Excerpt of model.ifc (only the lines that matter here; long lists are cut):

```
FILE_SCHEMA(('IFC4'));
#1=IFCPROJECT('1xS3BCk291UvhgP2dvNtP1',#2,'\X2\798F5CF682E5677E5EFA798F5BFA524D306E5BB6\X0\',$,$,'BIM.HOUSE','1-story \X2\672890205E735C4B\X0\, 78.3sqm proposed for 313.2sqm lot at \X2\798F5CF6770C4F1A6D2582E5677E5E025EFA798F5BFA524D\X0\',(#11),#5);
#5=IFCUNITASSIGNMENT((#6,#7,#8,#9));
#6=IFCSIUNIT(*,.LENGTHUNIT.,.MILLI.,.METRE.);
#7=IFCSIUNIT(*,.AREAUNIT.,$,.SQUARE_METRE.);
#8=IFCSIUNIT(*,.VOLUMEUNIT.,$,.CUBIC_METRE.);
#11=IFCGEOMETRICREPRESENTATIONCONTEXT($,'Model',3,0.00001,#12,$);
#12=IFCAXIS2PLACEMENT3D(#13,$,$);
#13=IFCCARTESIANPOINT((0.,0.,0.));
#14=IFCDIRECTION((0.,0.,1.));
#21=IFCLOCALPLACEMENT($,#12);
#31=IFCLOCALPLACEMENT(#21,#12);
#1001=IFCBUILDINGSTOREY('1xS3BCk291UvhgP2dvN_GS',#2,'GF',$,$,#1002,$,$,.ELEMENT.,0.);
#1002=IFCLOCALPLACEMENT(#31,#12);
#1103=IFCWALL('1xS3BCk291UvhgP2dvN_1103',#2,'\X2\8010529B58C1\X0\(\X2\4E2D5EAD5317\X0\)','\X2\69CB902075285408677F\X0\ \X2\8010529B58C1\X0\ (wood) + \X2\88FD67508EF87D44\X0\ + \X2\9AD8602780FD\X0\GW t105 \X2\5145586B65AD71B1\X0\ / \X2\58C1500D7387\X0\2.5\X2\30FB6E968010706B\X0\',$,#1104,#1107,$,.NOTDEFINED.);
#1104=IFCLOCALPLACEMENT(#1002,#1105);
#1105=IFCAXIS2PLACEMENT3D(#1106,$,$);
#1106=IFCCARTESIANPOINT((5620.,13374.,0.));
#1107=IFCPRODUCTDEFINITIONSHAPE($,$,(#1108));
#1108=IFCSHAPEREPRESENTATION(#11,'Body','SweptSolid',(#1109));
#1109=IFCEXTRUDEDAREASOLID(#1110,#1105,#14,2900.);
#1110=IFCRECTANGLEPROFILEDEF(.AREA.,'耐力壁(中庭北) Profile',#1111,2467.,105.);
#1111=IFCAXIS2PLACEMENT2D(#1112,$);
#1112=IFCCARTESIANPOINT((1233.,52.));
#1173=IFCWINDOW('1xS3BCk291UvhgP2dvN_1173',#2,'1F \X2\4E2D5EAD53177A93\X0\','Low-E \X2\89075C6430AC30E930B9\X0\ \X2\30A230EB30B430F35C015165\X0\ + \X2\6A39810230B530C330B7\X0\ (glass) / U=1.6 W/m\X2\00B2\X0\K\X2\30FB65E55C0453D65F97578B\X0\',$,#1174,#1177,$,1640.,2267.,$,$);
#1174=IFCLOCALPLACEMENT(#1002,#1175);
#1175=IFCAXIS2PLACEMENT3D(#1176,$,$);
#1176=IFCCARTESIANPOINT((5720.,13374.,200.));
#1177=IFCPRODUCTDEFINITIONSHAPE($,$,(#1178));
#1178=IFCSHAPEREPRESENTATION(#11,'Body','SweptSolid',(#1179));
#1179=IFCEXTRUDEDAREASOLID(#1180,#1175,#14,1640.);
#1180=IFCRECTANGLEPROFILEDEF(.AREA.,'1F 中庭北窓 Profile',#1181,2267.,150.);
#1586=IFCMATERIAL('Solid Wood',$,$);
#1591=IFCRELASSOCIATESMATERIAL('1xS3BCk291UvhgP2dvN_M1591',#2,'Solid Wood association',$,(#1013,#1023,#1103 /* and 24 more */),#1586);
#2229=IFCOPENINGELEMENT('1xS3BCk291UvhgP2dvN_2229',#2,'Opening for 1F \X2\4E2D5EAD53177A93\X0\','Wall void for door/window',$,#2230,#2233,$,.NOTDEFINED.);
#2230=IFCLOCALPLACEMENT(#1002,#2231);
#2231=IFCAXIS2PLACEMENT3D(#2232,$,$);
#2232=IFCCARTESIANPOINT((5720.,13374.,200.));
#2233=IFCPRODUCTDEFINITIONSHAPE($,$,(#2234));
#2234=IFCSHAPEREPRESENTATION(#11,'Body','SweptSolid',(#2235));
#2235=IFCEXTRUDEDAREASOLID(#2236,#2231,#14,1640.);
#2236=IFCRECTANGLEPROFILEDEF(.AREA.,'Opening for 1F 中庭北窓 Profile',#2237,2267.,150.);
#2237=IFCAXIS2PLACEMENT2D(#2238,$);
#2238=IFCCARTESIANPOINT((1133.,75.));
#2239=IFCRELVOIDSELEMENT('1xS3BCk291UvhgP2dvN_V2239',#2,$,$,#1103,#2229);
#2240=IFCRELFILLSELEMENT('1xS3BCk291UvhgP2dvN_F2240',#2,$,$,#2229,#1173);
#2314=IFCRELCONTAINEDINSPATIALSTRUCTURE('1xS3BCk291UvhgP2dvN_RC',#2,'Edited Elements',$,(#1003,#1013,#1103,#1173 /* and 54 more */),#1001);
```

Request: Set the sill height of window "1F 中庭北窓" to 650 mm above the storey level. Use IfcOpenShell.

```python
import numpy as np
import ifcopenshell
import ifcopenshell.api.geometry
import ifcopenshell.geom
import ifcopenshell.util.element
import ifcopenshell.util.placement
import ifcopenshell.util.shape
import ifcopenshell.util.unit

model = ifcopenshell.open("model.ifc")
unit_scale = ifcopenshell.util.unit.calculate_unit_scale(model)

window = model.by_guid("1xS3BCk291UvhgP2dvN_1173")
opening = window.FillsVoids[0].RelatingOpeningElement
storey = ifcopenshell.util.element.get_container(window, ifc_class="IfcBuildingStorey")
level = ifcopenshell.util.placement.get_local_placement(storey.ObjectPlacement)[2, 3]

# The opening's origin need not be at the sill, so measure its lowest point.
shape = ifcopenshell.geom.create_shape(ifcopenshell.geom.settings(), opening)
bottom = ifcopenshell.util.shape.get_shape_bottom_elevation(shape, shape.geometry) / unit_scale
dz = level + 0.65 / unit_scale - bottom

shift = np.array([0.0, 0.0, dz])
# The window is not placed relative to its opening, so move both.
for product in (opening, window):
    matrix = ifcopenshell.util.placement.get_local_placement(product.ObjectPlacement)
    matrix[:3, 3] += shift
    ifcopenshell.api.geometry.edit_object_placement(model, product=product, matrix=matrix, is_si=False)

print(f"moved by {dz * unit_scale:+.3f} m")

model.write("model_updated.ifc")
```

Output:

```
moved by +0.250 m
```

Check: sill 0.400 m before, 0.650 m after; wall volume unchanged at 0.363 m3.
